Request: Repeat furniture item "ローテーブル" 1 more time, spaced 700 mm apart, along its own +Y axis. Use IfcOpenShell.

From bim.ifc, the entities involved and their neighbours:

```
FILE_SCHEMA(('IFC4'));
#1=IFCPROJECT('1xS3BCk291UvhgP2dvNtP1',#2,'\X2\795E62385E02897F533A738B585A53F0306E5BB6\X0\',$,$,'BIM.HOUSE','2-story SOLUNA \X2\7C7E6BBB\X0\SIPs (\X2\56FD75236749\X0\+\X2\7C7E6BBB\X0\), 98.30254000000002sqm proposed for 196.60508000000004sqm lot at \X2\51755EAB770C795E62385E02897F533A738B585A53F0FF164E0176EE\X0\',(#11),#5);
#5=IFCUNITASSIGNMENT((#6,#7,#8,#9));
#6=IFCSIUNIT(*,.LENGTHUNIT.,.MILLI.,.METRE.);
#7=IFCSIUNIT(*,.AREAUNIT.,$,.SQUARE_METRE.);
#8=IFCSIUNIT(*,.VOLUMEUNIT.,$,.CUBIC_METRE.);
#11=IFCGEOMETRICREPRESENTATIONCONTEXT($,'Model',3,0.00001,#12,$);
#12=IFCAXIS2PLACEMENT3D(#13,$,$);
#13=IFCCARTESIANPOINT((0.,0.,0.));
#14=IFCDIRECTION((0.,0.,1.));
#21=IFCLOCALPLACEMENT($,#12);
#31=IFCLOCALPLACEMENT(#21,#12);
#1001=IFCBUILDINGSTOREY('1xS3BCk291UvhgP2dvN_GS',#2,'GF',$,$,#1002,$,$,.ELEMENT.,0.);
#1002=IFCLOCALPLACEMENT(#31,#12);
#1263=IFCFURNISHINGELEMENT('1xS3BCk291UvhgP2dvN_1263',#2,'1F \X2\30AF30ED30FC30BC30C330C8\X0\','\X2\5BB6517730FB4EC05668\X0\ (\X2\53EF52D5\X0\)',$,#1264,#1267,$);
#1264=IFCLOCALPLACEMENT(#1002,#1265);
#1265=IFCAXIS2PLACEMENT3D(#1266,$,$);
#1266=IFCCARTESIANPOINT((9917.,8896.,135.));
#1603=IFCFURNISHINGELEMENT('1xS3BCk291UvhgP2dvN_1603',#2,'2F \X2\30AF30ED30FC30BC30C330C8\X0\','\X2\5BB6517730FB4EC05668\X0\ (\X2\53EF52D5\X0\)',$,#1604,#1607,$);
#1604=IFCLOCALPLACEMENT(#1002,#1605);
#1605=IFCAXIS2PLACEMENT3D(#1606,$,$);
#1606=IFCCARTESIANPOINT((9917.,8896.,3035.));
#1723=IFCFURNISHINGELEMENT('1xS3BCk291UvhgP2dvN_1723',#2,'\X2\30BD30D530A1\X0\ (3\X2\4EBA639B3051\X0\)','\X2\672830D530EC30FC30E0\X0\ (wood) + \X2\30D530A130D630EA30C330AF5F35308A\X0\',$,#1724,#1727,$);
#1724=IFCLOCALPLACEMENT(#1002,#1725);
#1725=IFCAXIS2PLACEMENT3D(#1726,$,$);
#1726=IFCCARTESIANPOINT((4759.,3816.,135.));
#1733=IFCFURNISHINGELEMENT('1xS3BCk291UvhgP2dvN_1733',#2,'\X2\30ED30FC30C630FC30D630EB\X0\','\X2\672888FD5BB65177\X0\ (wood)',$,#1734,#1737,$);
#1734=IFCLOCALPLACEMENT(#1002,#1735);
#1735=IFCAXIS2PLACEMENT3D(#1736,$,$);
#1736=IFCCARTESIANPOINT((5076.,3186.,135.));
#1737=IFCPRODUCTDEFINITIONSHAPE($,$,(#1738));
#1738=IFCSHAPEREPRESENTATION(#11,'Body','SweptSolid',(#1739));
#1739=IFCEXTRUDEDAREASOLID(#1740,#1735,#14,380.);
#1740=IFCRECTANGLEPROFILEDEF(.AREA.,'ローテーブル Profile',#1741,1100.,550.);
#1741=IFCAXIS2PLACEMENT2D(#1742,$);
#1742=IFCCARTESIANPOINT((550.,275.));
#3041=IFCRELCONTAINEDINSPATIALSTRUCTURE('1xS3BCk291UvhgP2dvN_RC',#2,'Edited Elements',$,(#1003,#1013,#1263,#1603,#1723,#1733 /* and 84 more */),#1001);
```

```python
import ifcopenshell
import ifcopenshell.api.geometry
import ifcopenshell.api.root
import ifcopenshell.util.element
import ifcopenshell.util.placement

model = ifcopenshell.open("bim.ifc")


def reuse_history(source, copy):
    """copy_class also copies each property set's owner history, people and application; keep the originals."""
    for rel in copy.IsDefinedBy:
        if rel.is_a("IfcRelDefinesByProperties") and (history := rel.RelatingPropertyDefinition.OwnerHistory):
            rel.RelatingPropertyDefinition.OwnerHistory = source.OwnerHistory
            ifcopenshell.util.element.remove_deep2(model, history)


source = model.by_guid("1xS3BCk291UvhgP2dvN_1733")
base = ifcopenshell.util.placement.get_local_placement(source.ObjectPlacement)
step = base[:3, 1] * 700.0

for i in range(1, 2):
    copy = ifcopenshell.api.root.copy_class(model, product=source)
    copy.Representation = ifcopenshell.util.element.copy_deep(
        model, source.Representation, exclude=["IfcGeometricRepresentationContext", "IfcRepresentationMap"]
    )
    reuse_history(source, copy)
    matrix = base.copy()
    matrix[:3, 3] += i * step
    print("added at", matrix[:3, 3].round(3) + 0.0)
    ifcopenshell.api.geometry.edit_object_placement(model, product=copy, matrix=matrix, is_si=False)

model.write("bim_updated.ifc")
```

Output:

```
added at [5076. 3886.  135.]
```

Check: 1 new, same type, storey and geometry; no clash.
